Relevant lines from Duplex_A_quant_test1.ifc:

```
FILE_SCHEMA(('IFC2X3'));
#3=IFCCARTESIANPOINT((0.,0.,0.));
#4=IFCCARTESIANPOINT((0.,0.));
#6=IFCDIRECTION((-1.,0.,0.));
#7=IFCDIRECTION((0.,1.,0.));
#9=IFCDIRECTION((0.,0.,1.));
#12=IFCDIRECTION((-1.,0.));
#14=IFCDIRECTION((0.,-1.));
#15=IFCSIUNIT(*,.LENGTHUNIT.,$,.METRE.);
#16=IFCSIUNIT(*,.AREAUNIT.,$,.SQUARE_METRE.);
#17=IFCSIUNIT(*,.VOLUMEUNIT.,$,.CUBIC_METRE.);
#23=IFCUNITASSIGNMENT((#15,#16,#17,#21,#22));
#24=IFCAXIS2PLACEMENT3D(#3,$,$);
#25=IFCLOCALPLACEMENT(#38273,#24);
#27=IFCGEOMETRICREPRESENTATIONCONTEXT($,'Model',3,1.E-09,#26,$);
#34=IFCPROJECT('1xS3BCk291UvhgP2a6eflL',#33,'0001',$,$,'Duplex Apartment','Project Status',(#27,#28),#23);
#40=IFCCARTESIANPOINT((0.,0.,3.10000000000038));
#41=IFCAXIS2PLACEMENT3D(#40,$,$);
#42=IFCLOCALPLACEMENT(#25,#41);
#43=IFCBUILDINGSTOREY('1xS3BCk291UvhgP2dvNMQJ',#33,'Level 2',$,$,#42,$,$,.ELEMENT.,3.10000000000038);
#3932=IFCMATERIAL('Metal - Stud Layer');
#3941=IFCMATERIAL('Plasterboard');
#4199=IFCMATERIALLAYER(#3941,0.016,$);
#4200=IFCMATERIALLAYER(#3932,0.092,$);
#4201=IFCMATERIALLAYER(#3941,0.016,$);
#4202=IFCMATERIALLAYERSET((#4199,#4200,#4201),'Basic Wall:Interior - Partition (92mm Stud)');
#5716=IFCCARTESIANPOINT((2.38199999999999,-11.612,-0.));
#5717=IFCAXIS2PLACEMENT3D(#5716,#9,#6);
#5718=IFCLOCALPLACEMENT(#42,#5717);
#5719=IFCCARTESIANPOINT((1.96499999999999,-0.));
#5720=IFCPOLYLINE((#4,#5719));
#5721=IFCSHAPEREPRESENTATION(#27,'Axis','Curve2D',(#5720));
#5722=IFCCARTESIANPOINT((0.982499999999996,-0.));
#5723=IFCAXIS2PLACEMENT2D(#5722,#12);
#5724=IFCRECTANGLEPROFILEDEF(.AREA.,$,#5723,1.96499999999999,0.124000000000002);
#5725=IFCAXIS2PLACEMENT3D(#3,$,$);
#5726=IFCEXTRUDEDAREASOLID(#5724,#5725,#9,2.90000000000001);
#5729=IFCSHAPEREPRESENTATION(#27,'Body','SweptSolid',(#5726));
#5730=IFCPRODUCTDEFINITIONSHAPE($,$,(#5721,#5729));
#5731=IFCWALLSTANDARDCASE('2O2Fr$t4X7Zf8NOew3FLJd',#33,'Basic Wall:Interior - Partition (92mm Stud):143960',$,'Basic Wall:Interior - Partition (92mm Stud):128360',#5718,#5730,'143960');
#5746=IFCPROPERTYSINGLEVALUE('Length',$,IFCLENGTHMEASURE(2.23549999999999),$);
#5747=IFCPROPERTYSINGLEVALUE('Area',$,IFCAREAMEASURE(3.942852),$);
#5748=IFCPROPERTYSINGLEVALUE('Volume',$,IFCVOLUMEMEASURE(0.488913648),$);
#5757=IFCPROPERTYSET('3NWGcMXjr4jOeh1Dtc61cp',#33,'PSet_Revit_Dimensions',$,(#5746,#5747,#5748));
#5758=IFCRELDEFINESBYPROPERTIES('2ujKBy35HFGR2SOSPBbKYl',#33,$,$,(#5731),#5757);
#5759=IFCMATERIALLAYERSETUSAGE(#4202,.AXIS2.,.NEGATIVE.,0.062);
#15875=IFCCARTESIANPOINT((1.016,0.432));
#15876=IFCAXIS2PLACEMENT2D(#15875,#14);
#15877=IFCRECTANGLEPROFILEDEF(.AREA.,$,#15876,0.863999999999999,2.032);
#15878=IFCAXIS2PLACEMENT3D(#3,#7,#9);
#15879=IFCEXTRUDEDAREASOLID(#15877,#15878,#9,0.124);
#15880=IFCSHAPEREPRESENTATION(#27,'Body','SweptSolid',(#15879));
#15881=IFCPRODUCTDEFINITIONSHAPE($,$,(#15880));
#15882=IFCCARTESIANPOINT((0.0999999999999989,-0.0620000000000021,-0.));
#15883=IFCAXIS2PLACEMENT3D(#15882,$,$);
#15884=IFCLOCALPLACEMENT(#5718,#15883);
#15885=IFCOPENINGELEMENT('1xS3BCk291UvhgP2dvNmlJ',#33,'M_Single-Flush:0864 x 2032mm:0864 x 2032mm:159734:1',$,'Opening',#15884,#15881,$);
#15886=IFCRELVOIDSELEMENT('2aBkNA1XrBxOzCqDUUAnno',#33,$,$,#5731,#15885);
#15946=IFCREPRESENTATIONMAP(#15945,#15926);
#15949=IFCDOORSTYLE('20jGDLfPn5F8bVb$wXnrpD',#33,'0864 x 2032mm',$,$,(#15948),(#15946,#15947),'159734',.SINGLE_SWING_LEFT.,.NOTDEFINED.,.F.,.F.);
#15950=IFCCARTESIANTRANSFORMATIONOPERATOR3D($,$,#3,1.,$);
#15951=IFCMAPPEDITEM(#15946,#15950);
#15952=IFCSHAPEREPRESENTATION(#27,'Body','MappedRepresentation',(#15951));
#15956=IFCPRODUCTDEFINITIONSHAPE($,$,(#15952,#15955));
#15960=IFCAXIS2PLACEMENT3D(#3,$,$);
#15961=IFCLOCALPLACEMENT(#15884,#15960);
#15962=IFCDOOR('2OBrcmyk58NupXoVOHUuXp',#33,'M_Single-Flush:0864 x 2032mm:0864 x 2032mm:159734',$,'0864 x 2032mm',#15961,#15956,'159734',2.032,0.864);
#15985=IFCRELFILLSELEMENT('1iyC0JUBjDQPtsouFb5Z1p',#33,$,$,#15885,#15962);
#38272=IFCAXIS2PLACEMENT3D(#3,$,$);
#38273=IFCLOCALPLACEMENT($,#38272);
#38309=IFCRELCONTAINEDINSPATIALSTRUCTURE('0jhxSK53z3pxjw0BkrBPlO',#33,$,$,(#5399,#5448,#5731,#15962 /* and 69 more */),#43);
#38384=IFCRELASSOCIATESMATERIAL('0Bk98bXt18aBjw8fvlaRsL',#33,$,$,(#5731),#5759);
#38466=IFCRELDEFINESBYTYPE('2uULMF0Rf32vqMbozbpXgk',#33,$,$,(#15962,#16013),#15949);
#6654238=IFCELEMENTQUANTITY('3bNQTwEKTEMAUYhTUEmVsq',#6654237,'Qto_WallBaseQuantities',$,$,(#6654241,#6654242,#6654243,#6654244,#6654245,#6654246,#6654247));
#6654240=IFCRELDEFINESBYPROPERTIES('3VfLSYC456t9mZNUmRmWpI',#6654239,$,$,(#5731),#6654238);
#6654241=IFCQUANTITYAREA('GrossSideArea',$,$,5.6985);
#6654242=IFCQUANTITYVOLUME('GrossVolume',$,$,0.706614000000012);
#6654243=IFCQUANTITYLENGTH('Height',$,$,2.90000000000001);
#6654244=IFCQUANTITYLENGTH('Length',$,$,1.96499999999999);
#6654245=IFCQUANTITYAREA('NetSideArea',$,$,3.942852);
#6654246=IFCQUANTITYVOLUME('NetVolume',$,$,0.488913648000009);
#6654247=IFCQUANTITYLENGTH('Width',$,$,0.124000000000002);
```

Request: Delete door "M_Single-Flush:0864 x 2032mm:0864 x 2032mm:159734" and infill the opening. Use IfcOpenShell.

```python
import ifcopenshell
import ifcopenshell.api.feature
import ifcopenshell.api.pset
import ifcopenshell.api.root
import ifcopenshell.geom
import ifcopenshell.util.element
import ifcopenshell.util.shape
import ifcopenshell.util.unit

model = ifcopenshell.open("Duplex_A_quant_test1.ifc")
area_scale = ifcopenshell.util.unit.calculate_unit_scale(model, "AREAUNIT")
volume_scale = ifcopenshell.util.unit.calculate_unit_scale(model, "VOLUMEUNIT")
settings = ifcopenshell.geom.settings()


def volume(element):
    """Net volume in cubic metres, openings subtracted."""
    shape = ifcopenshell.geom.create_shape(settings, element)
    return ifcopenshell.util.shape.get_volume(shape.geometry)


door = model.by_guid("2OBrcmyk58NupXoVOHUuXp")
opening = door.FillsVoids[0].RelatingOpeningElement
wall = opening.VoidsElements[0].RelatingBuildingElement
before = volume(wall)

ifcopenshell.api.root.remove_product(model, product=door)
ifcopenshell.api.feature.remove_feature(model, feature=opening)

after = volume(wall)
thickness = 0.124  # wall thickness in metres

# Update the wall's stored quantities.
pset = model.by_id(ifcopenshell.util.element.get_pset(wall, "PSet_Revit_Dimensions", should_inherit=False)["id"])
ifcopenshell.api.pset.edit_pset(model, pset=pset, properties={
    "Area": model.create_entity("IfcAreaMeasure", after / thickness / area_scale),
    "Volume": model.create_entity("IfcVolumeMeasure", after / volume_scale),
})
qto = model.by_id(ifcopenshell.util.element.get_pset(wall, "Qto_WallBaseQuantities", should_inherit=False)["id"])
ifcopenshell.api.pset.edit_qto(model, qto=qto, properties={
    "NetSideArea": after / thickness / area_scale,
    "NetVolume": after / volume_scale,
})

print(f"wall volume {before:.3f} -> {after:.3f} m3")

model.write("Duplex_A_quant_test1_edited.ifc")
```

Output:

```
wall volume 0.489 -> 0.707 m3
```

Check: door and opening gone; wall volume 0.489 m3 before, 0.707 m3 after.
